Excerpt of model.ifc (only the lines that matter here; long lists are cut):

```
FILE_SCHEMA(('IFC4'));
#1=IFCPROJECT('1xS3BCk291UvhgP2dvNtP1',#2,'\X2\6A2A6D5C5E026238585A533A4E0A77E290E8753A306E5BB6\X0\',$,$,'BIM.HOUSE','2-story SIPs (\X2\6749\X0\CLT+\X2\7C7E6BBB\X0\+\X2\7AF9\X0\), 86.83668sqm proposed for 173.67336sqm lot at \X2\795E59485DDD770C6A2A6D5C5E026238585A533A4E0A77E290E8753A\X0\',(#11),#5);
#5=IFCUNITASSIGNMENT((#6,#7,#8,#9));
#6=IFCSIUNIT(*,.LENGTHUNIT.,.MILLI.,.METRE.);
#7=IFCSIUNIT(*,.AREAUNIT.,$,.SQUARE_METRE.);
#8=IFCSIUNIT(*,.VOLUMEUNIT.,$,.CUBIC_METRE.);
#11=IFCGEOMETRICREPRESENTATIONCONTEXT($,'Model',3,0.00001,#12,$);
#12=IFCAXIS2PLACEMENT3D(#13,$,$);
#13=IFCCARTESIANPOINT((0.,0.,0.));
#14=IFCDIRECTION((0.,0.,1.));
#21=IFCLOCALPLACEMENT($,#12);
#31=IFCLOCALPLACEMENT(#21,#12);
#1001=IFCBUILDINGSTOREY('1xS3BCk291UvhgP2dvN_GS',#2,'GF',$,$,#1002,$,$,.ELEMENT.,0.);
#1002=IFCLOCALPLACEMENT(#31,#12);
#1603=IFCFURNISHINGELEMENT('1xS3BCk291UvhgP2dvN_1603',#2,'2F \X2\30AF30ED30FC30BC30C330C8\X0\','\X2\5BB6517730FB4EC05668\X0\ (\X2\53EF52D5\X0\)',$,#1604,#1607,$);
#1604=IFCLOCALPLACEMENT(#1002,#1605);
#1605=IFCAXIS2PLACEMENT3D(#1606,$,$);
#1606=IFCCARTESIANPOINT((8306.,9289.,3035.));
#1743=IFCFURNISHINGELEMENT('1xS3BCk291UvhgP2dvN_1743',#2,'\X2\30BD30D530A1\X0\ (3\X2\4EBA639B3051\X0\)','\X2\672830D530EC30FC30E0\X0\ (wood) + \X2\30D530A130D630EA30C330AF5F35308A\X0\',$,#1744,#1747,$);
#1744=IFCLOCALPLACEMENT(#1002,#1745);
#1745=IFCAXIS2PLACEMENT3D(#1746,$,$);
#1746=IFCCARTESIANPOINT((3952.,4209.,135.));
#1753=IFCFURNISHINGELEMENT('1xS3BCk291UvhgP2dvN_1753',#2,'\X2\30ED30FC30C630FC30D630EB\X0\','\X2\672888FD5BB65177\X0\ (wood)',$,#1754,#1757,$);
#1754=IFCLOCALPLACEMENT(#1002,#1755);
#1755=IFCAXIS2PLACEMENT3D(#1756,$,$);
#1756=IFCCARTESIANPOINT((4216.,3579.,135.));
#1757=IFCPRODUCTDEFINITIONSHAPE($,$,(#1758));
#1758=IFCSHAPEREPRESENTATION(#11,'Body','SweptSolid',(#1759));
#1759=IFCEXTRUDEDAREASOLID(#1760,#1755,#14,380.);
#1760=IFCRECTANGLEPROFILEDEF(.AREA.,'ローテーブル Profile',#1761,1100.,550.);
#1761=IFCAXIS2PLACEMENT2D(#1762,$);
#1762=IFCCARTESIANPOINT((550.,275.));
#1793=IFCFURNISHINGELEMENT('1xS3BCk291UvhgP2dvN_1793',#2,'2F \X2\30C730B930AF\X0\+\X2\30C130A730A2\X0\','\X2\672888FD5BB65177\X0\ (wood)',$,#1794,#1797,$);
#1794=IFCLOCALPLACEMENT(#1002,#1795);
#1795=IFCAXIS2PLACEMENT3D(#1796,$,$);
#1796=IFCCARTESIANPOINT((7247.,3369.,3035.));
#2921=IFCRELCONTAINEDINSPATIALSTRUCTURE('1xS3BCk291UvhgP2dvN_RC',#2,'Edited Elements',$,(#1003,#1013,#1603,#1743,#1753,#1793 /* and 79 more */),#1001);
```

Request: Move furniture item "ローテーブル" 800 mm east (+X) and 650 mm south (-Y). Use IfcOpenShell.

```python
import ifcopenshell
import ifcopenshell.api.geometry
import ifcopenshell.util.placement
import ifcopenshell.util.unit

model = ifcopenshell.open("model.ifc")
unit_scale = ifcopenshell.util.unit.calculate_unit_scale(model)

item = model.by_guid("1xS3BCk291UvhgP2dvN_1753")
matrix = ifcopenshell.util.placement.get_local_placement(item.ObjectPlacement)
matrix[0, 3] += 0.8 / unit_scale
matrix[1, 3] -= 0.65 / unit_scale
ifcopenshell.api.geometry.edit_object_placement(model, product=item, matrix=matrix, is_si=False)

print(ifcopenshell.util.placement.get_local_placement(item.ObjectPlacement).round(3) + 0.0)

model.write("model_updated.ifc")
```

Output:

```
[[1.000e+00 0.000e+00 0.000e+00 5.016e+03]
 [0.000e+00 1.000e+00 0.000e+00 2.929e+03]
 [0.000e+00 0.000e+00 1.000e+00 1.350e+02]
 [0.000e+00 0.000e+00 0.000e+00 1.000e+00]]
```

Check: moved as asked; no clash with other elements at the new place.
